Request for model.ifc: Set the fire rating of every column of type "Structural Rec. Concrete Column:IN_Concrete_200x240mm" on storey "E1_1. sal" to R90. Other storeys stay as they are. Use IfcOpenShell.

First a look at what the model holds.

```python
import ifcopenshell
import ifcopenshell.util.element

model = ifcopenshell.open("model.ifc")
print(model.schema)
storey = next(s for s in model.by_type("IfcBuildingStorey") if s.Name == "E1_1. sal")
columns = [e for e in ifcopenshell.util.element.get_decomposition(storey) if e.is_a("IfcColumn")]
seen = {}
for e in columns:
    element_type = ifcopenshell.util.element.get_type(e)
    key = (element_type.Name if element_type != e and element_type else None, ifcopenshell.util.element.get_pset(e, "Pset_ColumnCommon", "FireRating"))
    seen[key] = seen.get(key, 0) + 1
for (name, value), count in sorted(seen.items(), key=str):
    print(count, "x", name, "|", value)
```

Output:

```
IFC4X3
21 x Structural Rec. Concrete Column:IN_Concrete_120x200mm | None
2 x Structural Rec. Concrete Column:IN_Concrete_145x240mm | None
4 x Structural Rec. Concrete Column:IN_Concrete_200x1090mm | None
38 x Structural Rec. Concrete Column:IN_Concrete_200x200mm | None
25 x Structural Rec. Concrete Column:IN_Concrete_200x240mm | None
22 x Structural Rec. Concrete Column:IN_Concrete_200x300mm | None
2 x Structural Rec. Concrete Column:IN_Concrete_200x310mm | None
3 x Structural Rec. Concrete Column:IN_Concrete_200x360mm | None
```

```python
import ifcopenshell
import ifcopenshell.api.pset
import ifcopenshell.util.element

model = ifcopenshell.open("model.ifc")

storey = next(s for s in model.by_type("IfcBuildingStorey") if s.Name == "E1_1. sal")
columns = [e for e in ifcopenshell.util.element.get_decomposition(storey) if e.is_a("IfcColumn")]

count = 0
for e in columns:
    element_type = ifcopenshell.util.element.get_type(e)
    if element_type in (None, e) or element_type.Name != "Structural Rec. Concrete Column:IN_Concrete_200x240mm":
        continue
    # add_pset returns the element's existing set when there is one.
    pset = ifcopenshell.api.pset.add_pset(model, product=e, name="Pset_ColumnCommon")
    ifcopenshell.api.pset.edit_pset(model, pset=pset, properties={"FireRating": "R90"})
    count += 1

print(count, "columns updated")

model.write("model_v2.ifc")
```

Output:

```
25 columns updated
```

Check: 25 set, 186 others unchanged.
